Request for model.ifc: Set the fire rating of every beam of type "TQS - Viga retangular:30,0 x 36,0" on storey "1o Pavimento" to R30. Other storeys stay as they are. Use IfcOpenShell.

First a look at what the model holds.

```python
import ifcopenshell
import ifcopenshell.util.element

model = ifcopenshell.open("model.ifc")
print(model.schema)
storey = next(s for s in model.by_type("IfcBuildingStorey") if s.Name == "1o Pavimento")
beams = [e for e in ifcopenshell.util.element.get_decomposition(storey) if e.is_a("IfcBeam")]
seen = {}
for e in beams:
    element_type = ifcopenshell.util.element.get_type(e)
    key = (element_type.Name if element_type != e and element_type else None, ifcopenshell.util.element.get_pset(e, "Pset_BeamCommon", "FireRating"))
    seen[key] = seen.get(key, 0) + 1
for (name, value), count in sorted(seen.items(), key=str):
    print(count, "x", name, "|", value)
```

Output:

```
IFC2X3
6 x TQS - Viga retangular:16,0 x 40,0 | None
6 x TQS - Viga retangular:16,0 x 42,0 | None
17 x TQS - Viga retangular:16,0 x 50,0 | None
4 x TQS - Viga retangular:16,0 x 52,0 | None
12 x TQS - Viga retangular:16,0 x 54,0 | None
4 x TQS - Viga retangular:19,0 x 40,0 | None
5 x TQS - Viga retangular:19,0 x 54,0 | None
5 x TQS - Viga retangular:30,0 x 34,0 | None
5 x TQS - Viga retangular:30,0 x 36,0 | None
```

```python
import ifcopenshell
import ifcopenshell.api.pset
import ifcopenshell.util.element

model = ifcopenshell.open("model.ifc")

storey = next(s for s in model.by_type("IfcBuildingStorey") if s.Name == "1o Pavimento")
beams = [e for e in ifcopenshell.util.element.get_decomposition(storey) if e.is_a("IfcBeam")]

count = 0
for e in beams:
    element_type = ifcopenshell.util.element.get_type(e)
    if element_type in (None, e) or element_type.Name != "TQS - Viga retangular:30,0 x 36,0":
        continue
    # add_pset returns the element's existing set when there is one.
    pset = ifcopenshell.api.pset.add_pset(model, product=e, name="Pset_BeamCommon")
    ifcopenshell.api.pset.edit_pset(model, pset=pset, properties={"FireRating": "R30"})
    count += 1

print(count, "beams updated")

model.write("model_rev.ifc")
```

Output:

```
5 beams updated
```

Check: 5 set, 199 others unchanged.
